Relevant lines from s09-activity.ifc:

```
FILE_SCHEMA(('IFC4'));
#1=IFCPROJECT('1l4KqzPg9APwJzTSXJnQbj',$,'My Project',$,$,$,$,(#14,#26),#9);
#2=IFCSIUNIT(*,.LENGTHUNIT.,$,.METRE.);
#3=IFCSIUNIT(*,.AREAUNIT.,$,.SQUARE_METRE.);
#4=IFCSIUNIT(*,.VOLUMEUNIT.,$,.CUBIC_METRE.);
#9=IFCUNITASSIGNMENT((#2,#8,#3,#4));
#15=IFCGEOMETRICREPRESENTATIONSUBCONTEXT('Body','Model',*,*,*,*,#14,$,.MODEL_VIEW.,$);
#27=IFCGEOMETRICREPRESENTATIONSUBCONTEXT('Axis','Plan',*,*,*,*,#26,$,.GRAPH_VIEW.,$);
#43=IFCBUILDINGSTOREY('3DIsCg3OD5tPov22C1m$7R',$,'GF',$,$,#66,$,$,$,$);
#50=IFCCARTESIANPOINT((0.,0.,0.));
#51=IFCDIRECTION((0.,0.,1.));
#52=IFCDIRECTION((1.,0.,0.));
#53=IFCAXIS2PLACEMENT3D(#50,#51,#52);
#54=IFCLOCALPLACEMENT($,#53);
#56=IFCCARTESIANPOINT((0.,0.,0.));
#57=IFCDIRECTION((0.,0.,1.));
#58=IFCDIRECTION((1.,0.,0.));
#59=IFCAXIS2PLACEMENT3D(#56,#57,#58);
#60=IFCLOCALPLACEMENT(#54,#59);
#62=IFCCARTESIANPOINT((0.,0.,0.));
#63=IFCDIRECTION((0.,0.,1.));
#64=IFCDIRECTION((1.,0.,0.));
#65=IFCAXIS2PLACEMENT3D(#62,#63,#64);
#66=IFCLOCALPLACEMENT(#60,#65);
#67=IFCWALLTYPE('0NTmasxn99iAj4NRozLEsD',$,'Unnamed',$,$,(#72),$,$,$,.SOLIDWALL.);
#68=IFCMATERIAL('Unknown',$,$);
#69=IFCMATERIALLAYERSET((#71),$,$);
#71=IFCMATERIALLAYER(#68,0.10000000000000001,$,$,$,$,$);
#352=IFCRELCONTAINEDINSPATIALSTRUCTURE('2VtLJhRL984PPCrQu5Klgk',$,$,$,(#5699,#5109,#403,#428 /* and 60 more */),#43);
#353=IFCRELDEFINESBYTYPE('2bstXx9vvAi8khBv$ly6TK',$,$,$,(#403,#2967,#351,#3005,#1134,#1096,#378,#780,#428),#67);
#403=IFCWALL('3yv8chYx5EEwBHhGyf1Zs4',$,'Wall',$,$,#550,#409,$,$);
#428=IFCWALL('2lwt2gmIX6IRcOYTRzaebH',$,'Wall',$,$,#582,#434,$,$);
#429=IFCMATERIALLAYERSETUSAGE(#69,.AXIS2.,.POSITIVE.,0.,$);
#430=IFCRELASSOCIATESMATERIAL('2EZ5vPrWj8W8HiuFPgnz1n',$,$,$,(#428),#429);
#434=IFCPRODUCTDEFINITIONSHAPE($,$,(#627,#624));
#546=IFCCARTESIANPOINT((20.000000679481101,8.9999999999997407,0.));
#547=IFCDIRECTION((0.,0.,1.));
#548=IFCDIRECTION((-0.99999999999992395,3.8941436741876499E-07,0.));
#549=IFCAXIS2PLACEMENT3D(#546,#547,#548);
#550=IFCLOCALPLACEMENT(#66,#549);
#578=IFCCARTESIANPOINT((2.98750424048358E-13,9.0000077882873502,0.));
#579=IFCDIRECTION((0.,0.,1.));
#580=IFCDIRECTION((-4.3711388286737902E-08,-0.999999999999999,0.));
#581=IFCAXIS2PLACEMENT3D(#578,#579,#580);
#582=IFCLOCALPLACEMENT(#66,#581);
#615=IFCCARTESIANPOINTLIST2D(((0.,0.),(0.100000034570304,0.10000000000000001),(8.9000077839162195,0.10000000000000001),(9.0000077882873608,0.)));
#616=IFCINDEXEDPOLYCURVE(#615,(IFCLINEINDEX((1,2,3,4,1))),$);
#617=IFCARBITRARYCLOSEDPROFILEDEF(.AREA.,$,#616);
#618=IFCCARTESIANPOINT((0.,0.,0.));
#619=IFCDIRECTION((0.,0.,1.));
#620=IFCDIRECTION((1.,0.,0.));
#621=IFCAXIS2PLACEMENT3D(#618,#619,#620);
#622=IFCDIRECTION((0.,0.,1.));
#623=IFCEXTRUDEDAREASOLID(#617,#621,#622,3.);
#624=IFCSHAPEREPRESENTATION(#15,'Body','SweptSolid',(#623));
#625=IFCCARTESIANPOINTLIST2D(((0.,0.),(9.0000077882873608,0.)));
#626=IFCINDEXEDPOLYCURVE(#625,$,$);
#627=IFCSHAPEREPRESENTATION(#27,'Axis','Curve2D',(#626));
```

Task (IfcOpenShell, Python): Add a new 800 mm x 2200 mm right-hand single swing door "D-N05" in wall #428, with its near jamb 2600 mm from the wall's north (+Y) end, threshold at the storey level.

```python
import numpy as np
import ifcopenshell
import ifcopenshell.api.feature
import ifcopenshell.api.geometry
import ifcopenshell.api.root
import ifcopenshell.api.spatial
import ifcopenshell.geom
import ifcopenshell.util.element
import ifcopenshell.util.placement
import ifcopenshell.util.representation
import ifcopenshell.util.shape
import ifcopenshell.util.unit

model = ifcopenshell.open("s09-activity.ifc")
unit_scale = ifcopenshell.util.unit.calculate_unit_scale(model)
settings = ifcopenshell.geom.settings()


def volume(element):
    """Net volume in cubic metres, openings subtracted."""
    shape = ifcopenshell.geom.create_shape(settings, element)
    return ifcopenshell.util.shape.get_volume(shape.geometry)


wall = model.by_id(428)
storey = ifcopenshell.util.element.get_container(wall, ifc_class="IfcBuildingStorey")
context = ifcopenshell.util.representation.get_context(model, "Model", "Body", "MODEL_VIEW")
before = volume(wall)

width, height, from_end, sill = 0.8, 2.2, 2.6, 0.0  # metres

# The wall runs along its own X axis, and the end named is its -X end.
wall_shape = ifcopenshell.geom.create_shape(settings, wall)
x, y, z = ifcopenshell.util.shape.get_vertices(wall_shape.geometry).T
start = x.min() + from_end
face, thickness = float(y.min()), float(y.max() - y.min())
wall_matrix = ifcopenshell.util.placement.get_local_placement(wall.ObjectPlacement)
level = ifcopenshell.util.placement.get_local_placement(storey.ObjectPlacement)[2, 3]


def in_wall(x, y):
    """Placement at x, y metres in the wall's axes, at sill height."""
    matrix = wall_matrix.copy()
    matrix[:, 3] = wall_matrix @ np.array([x / unit_scale, y / unit_scale, 0.0, 1.0])
    matrix[2, 3] = level + sill / unit_scale
    return matrix


# Opening: a box that overshoots both wall faces by 50 mm.
opening = ifcopenshell.api.root.create_entity(model, ifc_class="IfcOpeningElement", predefined_type="OPENING")
box = ifcopenshell.api.geometry.add_wall_representation(
    model, context=context, length=width, height=height, thickness=thickness + 0.1
)
ifcopenshell.api.geometry.assign_representation(model, product=opening, representation=box)
ifcopenshell.api.geometry.edit_object_placement(model, product=opening, matrix=in_wall(start, face - 0.05), is_si=False)
ifcopenshell.api.feature.add_feature(model, feature=opening, element=wall)

door = ifcopenshell.api.root.create_entity(model, ifc_class="IfcDoor", name="D-N05", predefined_type="DOOR")
door.OverallWidth, door.OverallHeight = width / unit_scale, height / unit_scale
door.OperationType = "SINGLE_SWING_RIGHT"
body = ifcopenshell.api.geometry.add_door_representation(
    model,
    context=context,
    overall_width=door.OverallWidth,
    overall_height=door.OverallHeight,
    operation_type="SINGLE_SWING_RIGHT",
    lining_properties={"LiningDepth": thickness / unit_scale, "ThresholdDepth": thickness / unit_scale},
)
ifcopenshell.api.geometry.assign_representation(model, product=door, representation=body)
ifcopenshell.api.spatial.assign_container(model, products=[door], relating_structure=storey)
ifcopenshell.api.feature.add_filling(model, opening=opening, element=door)

# The lining spans the wall, so the door starts at the wall face.
ifcopenshell.api.geometry.edit_object_placement(model, product=door, matrix=in_wall(start, face), is_si=False)

after = volume(wall)

print(f"wall volume {before:.3f} -> {after:.3f} m3")

model.write("s09-activity_v2.ifc")
```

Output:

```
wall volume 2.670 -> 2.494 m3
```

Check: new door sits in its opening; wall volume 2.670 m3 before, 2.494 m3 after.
